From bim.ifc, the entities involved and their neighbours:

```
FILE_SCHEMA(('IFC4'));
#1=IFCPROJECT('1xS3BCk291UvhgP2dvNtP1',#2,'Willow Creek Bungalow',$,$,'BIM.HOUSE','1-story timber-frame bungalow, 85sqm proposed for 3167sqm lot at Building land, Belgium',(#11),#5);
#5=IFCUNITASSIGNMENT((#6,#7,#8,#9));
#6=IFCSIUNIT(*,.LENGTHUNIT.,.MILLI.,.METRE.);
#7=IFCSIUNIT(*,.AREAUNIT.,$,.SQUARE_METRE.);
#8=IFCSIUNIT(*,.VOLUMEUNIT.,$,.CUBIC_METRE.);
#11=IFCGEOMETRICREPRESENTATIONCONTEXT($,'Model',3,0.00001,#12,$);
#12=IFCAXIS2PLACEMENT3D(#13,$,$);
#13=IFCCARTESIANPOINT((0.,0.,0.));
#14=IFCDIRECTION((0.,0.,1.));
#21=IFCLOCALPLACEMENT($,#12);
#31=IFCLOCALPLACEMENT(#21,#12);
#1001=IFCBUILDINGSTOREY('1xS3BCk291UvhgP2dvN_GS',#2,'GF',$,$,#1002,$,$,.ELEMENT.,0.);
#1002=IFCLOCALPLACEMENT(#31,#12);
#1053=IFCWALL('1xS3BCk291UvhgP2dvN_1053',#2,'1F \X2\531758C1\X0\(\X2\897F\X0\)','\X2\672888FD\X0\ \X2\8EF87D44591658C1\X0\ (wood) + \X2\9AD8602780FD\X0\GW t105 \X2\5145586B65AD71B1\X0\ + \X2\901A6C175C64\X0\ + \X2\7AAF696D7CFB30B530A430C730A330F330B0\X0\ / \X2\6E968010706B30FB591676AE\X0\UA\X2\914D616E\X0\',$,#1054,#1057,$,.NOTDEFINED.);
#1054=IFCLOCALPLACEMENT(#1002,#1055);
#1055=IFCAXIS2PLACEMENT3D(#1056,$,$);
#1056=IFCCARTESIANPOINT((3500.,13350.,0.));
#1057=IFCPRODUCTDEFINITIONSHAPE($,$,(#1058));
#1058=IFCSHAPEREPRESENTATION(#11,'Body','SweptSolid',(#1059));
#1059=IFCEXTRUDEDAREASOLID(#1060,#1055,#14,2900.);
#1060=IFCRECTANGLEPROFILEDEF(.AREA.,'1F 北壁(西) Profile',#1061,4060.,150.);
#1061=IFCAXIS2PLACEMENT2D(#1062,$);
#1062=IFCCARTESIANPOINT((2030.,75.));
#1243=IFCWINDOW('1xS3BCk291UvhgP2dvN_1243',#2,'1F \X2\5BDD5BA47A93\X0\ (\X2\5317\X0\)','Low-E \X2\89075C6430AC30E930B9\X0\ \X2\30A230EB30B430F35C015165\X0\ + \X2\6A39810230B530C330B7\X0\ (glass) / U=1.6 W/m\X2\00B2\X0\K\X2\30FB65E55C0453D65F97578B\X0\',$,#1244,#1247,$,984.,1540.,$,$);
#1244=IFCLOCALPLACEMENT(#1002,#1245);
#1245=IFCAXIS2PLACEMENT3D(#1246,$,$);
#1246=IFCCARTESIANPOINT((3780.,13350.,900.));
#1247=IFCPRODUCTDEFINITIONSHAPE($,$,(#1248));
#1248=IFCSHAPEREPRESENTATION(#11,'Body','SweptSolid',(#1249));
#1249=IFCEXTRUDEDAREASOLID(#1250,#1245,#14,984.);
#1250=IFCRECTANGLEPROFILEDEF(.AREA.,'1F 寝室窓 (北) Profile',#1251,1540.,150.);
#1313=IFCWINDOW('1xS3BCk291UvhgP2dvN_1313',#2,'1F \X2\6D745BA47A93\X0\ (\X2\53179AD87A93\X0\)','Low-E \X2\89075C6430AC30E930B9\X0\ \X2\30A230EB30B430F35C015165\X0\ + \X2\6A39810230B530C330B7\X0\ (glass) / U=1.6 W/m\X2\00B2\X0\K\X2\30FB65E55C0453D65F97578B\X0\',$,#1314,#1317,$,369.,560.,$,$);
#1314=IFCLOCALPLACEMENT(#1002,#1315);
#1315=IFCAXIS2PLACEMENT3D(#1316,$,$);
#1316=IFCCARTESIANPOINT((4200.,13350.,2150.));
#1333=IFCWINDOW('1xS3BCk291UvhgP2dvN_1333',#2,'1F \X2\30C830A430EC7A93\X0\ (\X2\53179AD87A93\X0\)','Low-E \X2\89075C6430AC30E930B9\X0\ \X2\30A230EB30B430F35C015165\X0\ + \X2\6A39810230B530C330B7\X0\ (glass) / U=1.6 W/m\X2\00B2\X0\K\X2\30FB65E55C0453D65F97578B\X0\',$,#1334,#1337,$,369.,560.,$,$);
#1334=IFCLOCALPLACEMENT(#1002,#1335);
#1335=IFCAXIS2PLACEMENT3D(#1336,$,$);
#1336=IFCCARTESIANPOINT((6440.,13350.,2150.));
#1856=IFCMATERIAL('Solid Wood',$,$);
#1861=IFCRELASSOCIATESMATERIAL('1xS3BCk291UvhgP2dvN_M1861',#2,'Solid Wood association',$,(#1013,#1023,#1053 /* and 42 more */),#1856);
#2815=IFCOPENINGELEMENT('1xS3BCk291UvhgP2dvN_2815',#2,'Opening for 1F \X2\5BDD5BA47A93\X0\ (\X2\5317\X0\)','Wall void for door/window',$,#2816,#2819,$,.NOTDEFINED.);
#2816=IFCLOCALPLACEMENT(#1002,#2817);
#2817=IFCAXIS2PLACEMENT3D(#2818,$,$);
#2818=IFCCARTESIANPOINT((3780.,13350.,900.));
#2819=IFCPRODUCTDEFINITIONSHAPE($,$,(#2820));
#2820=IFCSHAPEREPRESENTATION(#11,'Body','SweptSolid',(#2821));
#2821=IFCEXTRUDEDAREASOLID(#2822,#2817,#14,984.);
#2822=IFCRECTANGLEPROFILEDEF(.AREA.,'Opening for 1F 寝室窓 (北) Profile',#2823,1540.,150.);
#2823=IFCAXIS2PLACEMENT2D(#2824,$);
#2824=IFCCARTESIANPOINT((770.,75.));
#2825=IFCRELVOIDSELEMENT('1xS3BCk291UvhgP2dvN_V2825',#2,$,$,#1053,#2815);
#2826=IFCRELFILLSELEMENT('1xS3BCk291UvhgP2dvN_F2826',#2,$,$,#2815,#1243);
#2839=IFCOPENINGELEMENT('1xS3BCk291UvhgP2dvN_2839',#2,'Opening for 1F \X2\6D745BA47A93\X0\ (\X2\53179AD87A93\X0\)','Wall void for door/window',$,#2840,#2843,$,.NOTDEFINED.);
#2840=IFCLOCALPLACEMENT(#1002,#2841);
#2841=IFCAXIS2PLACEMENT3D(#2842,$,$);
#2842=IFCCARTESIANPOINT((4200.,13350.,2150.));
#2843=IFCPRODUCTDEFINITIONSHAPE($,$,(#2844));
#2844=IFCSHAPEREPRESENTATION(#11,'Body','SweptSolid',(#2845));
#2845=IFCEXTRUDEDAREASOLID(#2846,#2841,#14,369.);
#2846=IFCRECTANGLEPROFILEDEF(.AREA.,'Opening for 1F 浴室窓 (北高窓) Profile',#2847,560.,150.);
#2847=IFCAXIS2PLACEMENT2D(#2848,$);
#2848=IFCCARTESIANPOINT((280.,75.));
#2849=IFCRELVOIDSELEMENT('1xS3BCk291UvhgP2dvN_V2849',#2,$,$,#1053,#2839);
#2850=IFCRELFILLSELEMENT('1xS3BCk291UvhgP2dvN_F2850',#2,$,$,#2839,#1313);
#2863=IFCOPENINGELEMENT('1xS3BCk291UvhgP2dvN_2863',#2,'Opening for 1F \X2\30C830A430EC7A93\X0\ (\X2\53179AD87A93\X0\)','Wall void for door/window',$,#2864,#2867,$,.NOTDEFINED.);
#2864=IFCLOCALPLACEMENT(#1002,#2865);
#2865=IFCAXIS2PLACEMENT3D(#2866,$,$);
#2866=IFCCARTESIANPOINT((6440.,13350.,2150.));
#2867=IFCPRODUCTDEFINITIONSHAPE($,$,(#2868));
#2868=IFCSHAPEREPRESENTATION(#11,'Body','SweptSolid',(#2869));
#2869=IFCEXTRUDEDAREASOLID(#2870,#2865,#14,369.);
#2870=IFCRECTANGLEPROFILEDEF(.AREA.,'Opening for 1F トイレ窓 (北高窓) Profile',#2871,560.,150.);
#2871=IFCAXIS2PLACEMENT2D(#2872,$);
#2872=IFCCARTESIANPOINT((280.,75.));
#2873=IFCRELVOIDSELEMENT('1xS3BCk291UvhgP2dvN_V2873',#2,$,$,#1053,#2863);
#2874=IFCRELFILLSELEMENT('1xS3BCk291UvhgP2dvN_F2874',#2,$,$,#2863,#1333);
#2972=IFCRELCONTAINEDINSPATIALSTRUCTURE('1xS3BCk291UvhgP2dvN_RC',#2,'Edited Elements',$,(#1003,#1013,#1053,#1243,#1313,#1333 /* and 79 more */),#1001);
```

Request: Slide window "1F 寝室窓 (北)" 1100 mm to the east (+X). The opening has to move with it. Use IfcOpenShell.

```python
import ifcopenshell
import ifcopenshell.api.geometry
import ifcopenshell.util.placement
import ifcopenshell.util.unit

model = ifcopenshell.open("bim.ifc")
unit_scale = ifcopenshell.util.unit.calculate_unit_scale(model)

window = model.by_guid("1xS3BCk291UvhgP2dvN_1243")
opening = window.FillsVoids[0].RelatingOpeningElement
wall = opening.VoidsElements[0].RelatingBuildingElement

wall_matrix = ifcopenshell.util.placement.get_local_placement(wall.ObjectPlacement)
shift = wall_matrix[:3, 0] * 1.1 / unit_scale
before = ifcopenshell.util.placement.get_local_placement(window.ObjectPlacement)[:3, 3].copy()

# The window is not placed relative to its opening, so move both.
for product in (opening, window):
    matrix = ifcopenshell.util.placement.get_local_placement(product.ObjectPlacement)
    matrix[:3, 3] += shift
    ifcopenshell.api.geometry.edit_object_placement(model, product=product, matrix=matrix, is_si=False)

after = ifcopenshell.util.placement.get_local_placement(window.ObjectPlacement)[:3, 3]
print("window moved by", (after - before).round(3) + 0.0)

model.write("bim_v2.ifc")
```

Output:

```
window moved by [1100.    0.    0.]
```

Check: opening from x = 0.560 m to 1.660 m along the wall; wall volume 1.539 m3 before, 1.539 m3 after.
